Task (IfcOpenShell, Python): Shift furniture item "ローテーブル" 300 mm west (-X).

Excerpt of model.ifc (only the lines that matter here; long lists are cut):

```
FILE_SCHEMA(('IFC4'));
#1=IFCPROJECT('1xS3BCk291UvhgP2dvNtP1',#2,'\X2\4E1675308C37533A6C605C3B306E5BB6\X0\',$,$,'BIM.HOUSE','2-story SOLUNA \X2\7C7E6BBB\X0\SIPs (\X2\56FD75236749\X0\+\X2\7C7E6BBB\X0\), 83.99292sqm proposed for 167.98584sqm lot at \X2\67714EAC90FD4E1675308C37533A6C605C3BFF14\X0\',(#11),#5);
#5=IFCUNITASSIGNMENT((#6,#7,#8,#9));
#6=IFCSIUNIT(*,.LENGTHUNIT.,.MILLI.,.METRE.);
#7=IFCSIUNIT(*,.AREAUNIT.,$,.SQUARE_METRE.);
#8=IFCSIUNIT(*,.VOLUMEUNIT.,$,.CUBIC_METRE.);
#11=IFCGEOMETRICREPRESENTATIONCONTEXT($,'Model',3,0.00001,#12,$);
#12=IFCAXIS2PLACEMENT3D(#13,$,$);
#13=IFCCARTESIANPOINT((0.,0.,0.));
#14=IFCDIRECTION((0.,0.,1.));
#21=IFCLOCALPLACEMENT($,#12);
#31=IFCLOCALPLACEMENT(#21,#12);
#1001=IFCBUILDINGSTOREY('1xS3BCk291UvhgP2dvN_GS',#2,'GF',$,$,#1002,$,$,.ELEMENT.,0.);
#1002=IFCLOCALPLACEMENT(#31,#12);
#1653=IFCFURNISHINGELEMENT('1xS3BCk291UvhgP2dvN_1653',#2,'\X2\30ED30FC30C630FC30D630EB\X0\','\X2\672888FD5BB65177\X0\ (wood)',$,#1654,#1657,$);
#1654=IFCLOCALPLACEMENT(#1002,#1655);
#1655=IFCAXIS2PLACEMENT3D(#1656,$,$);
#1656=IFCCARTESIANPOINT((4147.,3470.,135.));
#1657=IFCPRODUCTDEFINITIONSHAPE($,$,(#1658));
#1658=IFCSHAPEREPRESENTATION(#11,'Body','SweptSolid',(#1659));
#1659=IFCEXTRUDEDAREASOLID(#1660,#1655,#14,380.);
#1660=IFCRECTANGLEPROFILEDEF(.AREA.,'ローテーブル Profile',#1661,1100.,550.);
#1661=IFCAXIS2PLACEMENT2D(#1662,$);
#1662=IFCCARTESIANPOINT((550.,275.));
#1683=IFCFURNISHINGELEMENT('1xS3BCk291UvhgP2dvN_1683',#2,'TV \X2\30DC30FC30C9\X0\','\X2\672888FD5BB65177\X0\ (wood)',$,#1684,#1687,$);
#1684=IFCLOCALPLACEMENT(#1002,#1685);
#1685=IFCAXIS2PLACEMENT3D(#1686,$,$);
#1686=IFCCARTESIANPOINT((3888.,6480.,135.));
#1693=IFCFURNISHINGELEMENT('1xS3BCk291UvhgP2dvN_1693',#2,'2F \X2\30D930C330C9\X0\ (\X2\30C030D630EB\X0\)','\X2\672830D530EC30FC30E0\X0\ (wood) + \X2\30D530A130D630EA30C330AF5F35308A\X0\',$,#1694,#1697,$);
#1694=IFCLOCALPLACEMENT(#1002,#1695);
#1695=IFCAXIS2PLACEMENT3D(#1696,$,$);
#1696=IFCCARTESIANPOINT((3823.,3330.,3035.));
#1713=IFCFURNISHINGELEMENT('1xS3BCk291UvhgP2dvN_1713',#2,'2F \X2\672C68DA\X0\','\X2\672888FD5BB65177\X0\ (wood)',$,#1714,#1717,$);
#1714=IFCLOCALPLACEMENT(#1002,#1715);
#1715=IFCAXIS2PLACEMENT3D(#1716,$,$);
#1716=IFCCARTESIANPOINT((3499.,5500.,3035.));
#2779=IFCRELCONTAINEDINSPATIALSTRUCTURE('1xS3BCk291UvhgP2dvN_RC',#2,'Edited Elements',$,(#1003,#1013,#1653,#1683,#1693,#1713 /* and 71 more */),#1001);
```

```python
import ifcopenshell
import ifcopenshell.api.geometry
import ifcopenshell.util.placement

model = ifcopenshell.open("model.ifc")

item = model.by_guid("1xS3BCk291UvhgP2dvN_1653")
matrix = ifcopenshell.util.placement.get_local_placement(item.ObjectPlacement)
matrix[0, 3] -= 300.0
ifcopenshell.api.geometry.edit_object_placement(model, product=item, matrix=matrix, is_si=False)

print(ifcopenshell.util.placement.get_local_placement(item.ObjectPlacement).round(3) + 0.0)

model.write("model_updated.ifc")
```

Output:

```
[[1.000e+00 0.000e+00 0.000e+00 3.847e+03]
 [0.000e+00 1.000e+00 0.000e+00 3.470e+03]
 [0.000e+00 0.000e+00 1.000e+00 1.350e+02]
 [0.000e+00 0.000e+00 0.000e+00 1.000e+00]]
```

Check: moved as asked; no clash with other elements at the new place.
